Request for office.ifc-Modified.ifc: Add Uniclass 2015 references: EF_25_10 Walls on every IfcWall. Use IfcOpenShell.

First a look at what the model holds.

```python
import ifcopenshell

model = ifcopenshell.open("office.ifc-Modified.ifc")
print(model.schema)
print("classifications:", [c.Name for c in model.by_type("IfcClassification")])
for ifc_class in ("IfcDoor", "IfcRoof", "IfcStair", "IfcWall", "IfcWindow"):
    print(ifc_class, len(model.by_type(ifc_class)))
```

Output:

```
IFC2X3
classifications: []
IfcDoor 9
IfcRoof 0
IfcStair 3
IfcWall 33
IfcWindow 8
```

```python
import ifcopenshell
import ifcopenshell.api.classification

model = ifcopenshell.open("office.ifc-Modified.ifc")

# IFC2X3 requires Source and Edition and has no link from the project to the system.
system = model.create_entity("IfcClassification", Source="NBS", Edition="2015", Name="Uniclass 2015")

codes = {
    "IfcWall": ("EF_25_10", "Walls"),
}
for ifc_class, (code, name) in codes.items():
    products = model.by_type(ifc_class)
    ifcopenshell.api.classification.add_reference(
        model, products=products, classification=system, identification=code, name=name
    )
    print(code, len(products))

model.write("office.ifc-Modified-out.ifc")
```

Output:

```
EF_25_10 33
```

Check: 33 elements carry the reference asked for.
